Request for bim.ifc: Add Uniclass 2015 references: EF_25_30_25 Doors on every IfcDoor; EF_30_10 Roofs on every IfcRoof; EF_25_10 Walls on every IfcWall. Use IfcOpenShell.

First a look at what the model holds.

```python
import ifcopenshell

model = ifcopenshell.open("bim.ifc")
print(model.schema)
print("classifications:", [c.Name for c in model.by_type("IfcClassification")])
for ifc_class in ("IfcDoor", "IfcRoof", "IfcStair", "IfcWall", "IfcWindow"):
    print(ifc_class, len(model.by_type(ifc_class)))
```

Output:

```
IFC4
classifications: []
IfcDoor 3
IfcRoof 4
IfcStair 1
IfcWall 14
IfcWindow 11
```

```python
import ifcopenshell
import ifcopenshell.api.classification

model = ifcopenshell.open("bim.ifc")

system = ifcopenshell.api.classification.add_classification(model, classification="Uniclass 2015")

codes = {
    "IfcDoor": ("EF_25_30_25", "Doors"),
    "IfcRoof": ("EF_30_10", "Roofs"),
    "IfcWall": ("EF_25_10", "Walls"),
}
for ifc_class, (code, name) in codes.items():
    products = model.by_type(ifc_class)
    ifcopenshell.api.classification.add_reference(
        model, products=products, classification=system, identification=code, name=name
    )
    print(code, len(products))

model.write("bim_rev.ifc")
```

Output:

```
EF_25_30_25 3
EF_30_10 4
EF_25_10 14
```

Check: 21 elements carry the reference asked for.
